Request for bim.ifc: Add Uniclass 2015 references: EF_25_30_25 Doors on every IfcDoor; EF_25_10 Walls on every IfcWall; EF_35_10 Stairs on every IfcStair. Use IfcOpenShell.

First a look at what the model holds.

```python
import ifcopenshell

model = ifcopenshell.open("bim.ifc")
print(model.schema)
print("classifications:", [c.Name for c in model.by_type("IfcClassification")])
for ifc_class in ("IfcDoor", "IfcRoof", "IfcStair", "IfcWall", "IfcWindow"):
    print(ifc_class, len(model.by_type(ifc_class)))
```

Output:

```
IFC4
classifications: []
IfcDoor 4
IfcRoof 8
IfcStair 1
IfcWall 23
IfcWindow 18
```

```python
import ifcopenshell
import ifcopenshell.api.classification

model = ifcopenshell.open("bim.ifc")

system = ifcopenshell.api.classification.add_classification(model, classification="Uniclass 2015")

codes = {
    "IfcDoor": ("EF_25_30_25", "Doors"),
    "IfcWall": ("EF_25_10", "Walls"),
    "IfcStair": ("EF_35_10", "Stairs"),
}
for ifc_class, (code, name) in codes.items():
    products = model.by_type(ifc_class)
    ifcopenshell.api.classification.add_reference(
        model, products=products, classification=system, identification=code, name=name
    )
    print(code, len(products))

model.write("bim_edited.ifc")
```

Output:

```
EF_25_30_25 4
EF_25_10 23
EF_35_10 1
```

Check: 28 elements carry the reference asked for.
